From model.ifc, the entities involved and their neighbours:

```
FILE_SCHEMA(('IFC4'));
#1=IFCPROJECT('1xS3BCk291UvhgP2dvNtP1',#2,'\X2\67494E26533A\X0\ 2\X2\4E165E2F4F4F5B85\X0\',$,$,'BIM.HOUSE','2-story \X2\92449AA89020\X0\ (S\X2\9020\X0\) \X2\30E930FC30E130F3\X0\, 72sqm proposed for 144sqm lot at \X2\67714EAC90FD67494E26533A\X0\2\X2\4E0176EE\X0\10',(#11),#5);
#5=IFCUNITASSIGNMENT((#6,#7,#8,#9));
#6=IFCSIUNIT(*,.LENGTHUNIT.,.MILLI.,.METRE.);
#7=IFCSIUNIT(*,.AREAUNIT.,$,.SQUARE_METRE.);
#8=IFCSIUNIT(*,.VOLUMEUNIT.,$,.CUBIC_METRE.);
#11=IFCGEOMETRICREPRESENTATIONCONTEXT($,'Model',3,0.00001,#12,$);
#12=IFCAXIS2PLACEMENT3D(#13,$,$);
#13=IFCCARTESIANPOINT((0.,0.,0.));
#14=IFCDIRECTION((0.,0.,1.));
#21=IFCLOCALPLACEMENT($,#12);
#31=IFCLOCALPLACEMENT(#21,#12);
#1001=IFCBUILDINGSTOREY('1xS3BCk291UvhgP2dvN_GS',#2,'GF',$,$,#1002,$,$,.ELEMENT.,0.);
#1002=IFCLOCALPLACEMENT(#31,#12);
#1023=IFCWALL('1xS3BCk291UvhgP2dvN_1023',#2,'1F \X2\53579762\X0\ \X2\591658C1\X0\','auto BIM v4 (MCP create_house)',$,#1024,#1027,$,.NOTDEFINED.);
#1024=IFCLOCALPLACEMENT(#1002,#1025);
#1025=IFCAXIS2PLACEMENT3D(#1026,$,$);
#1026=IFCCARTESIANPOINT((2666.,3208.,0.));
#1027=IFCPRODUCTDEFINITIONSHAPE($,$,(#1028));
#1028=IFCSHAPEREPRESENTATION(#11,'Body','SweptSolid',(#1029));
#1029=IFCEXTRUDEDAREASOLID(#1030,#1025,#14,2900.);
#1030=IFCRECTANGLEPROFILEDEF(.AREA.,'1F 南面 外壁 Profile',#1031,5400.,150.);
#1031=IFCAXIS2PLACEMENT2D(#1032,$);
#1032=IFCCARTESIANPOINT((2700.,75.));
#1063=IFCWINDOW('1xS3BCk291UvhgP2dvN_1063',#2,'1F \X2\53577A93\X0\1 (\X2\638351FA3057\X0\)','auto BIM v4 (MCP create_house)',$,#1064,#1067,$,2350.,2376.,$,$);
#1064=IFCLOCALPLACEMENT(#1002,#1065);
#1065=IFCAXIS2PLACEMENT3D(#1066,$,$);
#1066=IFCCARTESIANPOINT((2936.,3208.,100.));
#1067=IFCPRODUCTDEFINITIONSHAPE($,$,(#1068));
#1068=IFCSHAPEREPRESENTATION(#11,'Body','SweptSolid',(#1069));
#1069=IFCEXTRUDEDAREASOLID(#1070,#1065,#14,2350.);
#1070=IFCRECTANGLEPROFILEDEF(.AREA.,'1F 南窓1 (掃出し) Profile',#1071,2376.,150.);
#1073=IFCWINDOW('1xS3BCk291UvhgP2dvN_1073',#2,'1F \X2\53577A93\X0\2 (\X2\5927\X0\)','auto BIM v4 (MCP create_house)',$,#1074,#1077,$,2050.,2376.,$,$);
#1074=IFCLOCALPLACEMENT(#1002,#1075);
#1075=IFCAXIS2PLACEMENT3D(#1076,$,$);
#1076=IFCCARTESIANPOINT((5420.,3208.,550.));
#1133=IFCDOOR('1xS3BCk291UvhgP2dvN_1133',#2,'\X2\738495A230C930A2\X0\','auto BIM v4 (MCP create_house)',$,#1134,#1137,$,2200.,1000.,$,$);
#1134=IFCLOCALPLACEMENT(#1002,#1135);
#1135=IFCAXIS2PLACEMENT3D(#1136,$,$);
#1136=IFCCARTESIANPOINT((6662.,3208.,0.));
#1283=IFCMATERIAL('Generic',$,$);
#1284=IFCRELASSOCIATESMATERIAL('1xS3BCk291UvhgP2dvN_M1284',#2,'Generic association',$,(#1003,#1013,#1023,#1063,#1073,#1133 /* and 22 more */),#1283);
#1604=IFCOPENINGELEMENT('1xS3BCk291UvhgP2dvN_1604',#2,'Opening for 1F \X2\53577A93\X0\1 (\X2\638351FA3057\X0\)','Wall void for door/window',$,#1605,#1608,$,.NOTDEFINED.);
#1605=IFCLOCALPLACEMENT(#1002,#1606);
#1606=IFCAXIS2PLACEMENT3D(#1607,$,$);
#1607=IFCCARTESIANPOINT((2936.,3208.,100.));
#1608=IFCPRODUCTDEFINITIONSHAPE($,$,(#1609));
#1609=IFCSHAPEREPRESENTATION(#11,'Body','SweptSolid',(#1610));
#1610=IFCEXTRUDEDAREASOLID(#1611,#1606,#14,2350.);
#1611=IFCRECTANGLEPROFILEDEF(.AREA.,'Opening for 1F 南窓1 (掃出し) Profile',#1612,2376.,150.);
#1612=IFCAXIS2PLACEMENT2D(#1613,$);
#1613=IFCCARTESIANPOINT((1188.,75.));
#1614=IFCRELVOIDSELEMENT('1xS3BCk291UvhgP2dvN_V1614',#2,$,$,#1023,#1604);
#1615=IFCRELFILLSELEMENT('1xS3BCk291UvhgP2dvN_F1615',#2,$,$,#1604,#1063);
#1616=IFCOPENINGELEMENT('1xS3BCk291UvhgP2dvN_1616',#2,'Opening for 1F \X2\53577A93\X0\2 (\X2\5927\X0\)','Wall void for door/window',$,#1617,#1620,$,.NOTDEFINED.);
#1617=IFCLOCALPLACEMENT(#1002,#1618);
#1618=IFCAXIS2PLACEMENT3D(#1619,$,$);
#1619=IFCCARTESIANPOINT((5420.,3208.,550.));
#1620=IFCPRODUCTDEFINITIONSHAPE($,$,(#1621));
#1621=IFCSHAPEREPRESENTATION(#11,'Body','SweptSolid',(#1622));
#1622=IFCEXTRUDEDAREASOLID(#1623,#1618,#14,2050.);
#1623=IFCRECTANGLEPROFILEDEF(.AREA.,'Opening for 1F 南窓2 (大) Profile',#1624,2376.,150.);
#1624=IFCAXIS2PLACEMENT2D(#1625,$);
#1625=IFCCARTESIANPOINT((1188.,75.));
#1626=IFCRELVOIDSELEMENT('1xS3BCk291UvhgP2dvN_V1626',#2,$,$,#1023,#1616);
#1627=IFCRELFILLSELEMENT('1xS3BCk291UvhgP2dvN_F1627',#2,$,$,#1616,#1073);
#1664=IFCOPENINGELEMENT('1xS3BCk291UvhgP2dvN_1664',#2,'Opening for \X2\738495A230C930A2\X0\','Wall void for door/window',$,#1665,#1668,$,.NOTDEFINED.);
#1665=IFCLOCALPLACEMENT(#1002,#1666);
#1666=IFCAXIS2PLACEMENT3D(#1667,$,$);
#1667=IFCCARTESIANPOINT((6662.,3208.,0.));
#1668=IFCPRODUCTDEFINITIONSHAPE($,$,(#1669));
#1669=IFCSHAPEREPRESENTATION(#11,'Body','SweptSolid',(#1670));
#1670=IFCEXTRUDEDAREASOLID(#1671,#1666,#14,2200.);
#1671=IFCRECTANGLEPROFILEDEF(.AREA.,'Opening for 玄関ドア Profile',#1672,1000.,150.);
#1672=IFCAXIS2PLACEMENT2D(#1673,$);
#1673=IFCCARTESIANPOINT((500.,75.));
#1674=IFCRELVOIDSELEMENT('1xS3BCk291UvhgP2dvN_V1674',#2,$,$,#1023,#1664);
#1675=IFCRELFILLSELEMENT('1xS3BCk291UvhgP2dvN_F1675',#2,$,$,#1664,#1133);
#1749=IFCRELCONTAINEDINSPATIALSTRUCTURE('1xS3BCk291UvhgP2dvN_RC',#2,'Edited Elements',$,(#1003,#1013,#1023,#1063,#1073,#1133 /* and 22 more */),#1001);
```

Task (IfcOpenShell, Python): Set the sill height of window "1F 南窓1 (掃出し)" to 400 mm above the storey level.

```python
import numpy as np
import ifcopenshell
import ifcopenshell.api.geometry
import ifcopenshell.geom
import ifcopenshell.util.element
import ifcopenshell.util.placement
import ifcopenshell.util.shape
import ifcopenshell.util.unit

model = ifcopenshell.open("model.ifc")
unit_scale = ifcopenshell.util.unit.calculate_unit_scale(model)

window = model.by_guid("1xS3BCk291UvhgP2dvN_1063")
opening = window.FillsVoids[0].RelatingOpeningElement
storey = ifcopenshell.util.element.get_container(window, ifc_class="IfcBuildingStorey")
level = ifcopenshell.util.placement.get_local_placement(storey.ObjectPlacement)[2, 3]

# The opening's origin need not be at the sill, so measure its lowest point.
shape = ifcopenshell.geom.create_shape(ifcopenshell.geom.settings(), opening)
bottom = ifcopenshell.util.shape.get_shape_bottom_elevation(shape, shape.geometry) / unit_scale
dz = level + 0.4 / unit_scale - bottom

shift = np.array([0.0, 0.0, dz])
# The window is not placed relative to its opening, so move both.
for product in (opening, window):
    matrix = ifcopenshell.util.placement.get_local_placement(product.ObjectPlacement)
    matrix[:3, 3] += shift
    ifcopenshell.api.geometry.edit_object_placement(model, product=product, matrix=matrix, is_si=False)

print(f"moved by {dz * unit_scale:+.3f} m")

model.write("model_v2.ifc")
```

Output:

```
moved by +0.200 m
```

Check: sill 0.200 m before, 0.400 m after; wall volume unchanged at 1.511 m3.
